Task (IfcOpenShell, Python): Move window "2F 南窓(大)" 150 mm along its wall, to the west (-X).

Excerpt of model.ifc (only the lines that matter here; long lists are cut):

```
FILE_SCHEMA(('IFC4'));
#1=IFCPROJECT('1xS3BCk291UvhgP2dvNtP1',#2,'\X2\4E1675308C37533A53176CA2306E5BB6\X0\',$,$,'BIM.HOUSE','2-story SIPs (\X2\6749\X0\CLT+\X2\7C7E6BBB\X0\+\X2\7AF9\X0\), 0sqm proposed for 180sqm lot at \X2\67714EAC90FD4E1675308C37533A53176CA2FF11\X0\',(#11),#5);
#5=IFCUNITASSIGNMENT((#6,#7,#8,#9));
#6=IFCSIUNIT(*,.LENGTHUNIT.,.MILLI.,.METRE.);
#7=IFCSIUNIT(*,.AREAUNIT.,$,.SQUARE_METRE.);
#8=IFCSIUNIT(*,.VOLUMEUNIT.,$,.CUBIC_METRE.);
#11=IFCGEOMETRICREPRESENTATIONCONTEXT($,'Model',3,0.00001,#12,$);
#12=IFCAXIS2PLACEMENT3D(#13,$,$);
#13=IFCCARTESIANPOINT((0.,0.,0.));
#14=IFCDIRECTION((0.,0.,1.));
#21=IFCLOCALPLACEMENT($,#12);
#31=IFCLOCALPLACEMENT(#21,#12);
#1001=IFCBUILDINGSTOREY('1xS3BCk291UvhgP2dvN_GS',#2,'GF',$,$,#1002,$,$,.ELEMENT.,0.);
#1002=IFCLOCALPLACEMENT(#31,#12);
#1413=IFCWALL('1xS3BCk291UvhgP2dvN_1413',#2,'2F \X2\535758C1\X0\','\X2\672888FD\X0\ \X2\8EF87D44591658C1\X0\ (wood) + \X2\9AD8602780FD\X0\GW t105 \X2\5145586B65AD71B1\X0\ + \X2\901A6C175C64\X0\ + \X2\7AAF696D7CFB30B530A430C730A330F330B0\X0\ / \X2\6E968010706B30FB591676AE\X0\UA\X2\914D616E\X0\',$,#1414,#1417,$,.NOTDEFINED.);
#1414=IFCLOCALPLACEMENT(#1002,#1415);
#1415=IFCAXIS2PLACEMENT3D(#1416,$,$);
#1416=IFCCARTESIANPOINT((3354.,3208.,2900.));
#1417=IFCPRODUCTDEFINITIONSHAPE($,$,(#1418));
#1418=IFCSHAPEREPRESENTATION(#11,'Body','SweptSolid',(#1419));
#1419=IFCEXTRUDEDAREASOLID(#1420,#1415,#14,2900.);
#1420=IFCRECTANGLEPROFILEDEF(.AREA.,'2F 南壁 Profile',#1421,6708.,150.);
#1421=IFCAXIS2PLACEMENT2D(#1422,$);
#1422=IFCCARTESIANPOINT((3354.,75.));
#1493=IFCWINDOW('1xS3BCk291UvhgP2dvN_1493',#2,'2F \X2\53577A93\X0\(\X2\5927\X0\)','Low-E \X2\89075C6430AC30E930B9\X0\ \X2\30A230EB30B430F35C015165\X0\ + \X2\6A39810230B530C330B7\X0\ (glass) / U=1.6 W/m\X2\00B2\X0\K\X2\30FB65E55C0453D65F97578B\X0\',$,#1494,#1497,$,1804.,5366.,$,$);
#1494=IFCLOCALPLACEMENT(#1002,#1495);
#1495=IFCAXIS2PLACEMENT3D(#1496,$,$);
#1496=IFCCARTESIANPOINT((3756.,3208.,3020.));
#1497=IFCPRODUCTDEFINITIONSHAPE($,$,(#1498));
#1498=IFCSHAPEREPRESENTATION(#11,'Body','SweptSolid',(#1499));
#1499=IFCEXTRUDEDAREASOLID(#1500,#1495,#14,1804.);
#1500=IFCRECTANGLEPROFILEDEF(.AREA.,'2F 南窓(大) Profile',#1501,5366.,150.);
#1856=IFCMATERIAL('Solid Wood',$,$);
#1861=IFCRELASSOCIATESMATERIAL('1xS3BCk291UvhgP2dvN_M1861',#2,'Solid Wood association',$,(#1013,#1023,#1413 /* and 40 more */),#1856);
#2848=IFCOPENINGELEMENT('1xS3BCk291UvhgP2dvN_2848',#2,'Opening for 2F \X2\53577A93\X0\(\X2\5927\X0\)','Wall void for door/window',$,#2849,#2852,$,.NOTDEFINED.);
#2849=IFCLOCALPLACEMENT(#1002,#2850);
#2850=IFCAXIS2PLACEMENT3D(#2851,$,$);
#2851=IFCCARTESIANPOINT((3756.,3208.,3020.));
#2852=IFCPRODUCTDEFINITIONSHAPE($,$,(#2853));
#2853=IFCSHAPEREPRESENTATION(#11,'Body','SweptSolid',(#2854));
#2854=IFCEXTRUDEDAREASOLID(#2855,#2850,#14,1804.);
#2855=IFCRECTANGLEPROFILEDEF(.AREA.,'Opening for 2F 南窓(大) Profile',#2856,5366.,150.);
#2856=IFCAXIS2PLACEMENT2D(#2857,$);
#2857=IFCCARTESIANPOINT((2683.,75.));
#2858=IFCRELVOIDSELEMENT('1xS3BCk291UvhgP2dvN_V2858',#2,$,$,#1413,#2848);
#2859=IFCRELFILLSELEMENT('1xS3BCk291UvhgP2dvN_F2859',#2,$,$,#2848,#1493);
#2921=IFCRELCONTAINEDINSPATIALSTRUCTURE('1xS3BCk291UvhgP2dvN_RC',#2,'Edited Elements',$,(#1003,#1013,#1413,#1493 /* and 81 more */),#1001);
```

```python
import ifcopenshell
import ifcopenshell.api.geometry
import ifcopenshell.util.placement

model = ifcopenshell.open("model.ifc")

window = model.by_guid("1xS3BCk291UvhgP2dvN_1493")
opening = window.FillsVoids[0].RelatingOpeningElement
wall = opening.VoidsElements[0].RelatingBuildingElement

wall_matrix = ifcopenshell.util.placement.get_local_placement(wall.ObjectPlacement)
shift = wall_matrix[:3, 0] * -150.0
before = ifcopenshell.util.placement.get_local_placement(window.ObjectPlacement)[:3, 3].copy()

# The window is not placed relative to its opening, so move both.
for product in (opening, window):
    matrix = ifcopenshell.util.placement.get_local_placement(product.ObjectPlacement)
    matrix[:3, 3] += shift
    ifcopenshell.api.geometry.edit_object_placement(model, product=product, matrix=matrix, is_si=False)

after = ifcopenshell.util.placement.get_local_placement(window.ObjectPlacement)[:3, 3]
print("window moved by", (after - before).round(3) + 0.0)

model.write("model_v2.ifc")
```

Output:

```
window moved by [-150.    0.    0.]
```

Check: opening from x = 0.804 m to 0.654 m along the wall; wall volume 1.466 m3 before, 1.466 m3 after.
